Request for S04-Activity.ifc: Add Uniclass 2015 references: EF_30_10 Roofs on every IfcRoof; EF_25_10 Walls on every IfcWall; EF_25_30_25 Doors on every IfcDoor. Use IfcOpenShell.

First a look at what the model holds.

```python
import ifcopenshell

model = ifcopenshell.open("S04-Activity.ifc")
print(model.schema)
print("classifications:", [c.Name for c in model.by_type("IfcClassification")])
for ifc_class in ("IfcDoor", "IfcRoof", "IfcStair", "IfcWall", "IfcWindow"):
    print(ifc_class, len(model.by_type(ifc_class)))
```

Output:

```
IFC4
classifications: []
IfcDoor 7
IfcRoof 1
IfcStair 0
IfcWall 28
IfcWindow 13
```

```python
import ifcopenshell
import ifcopenshell.api.classification

model = ifcopenshell.open("S04-Activity.ifc")

system = ifcopenshell.api.classification.add_classification(model, classification="Uniclass 2015")

codes = {
    "IfcRoof": ("EF_30_10", "Roofs"),
    "IfcWall": ("EF_25_10", "Walls"),
    "IfcDoor": ("EF_25_30_25", "Doors"),
}
for ifc_class, (code, name) in codes.items():
    products = model.by_type(ifc_class)
    ifcopenshell.api.classification.add_reference(
        model, products=products, classification=system, identification=code, name=name
    )
    print(code, len(products))

model.write("S04-Activity_v2.ifc")
```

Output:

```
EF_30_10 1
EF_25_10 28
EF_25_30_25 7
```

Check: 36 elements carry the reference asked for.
